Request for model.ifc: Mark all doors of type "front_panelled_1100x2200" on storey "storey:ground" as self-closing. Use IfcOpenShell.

First a look at what the model holds.

```python
import ifcopenshell
import ifcopenshell.util.element

model = ifcopenshell.open("model.ifc")
print(model.schema)
storey = next(s for s in model.by_type("IfcBuildingStorey") if s.Name == "storey:ground")
doors = [e for e in ifcopenshell.util.element.get_decomposition(storey) if e.is_a("IfcDoor")]
seen = {}
for e in doors:
    element_type = ifcopenshell.util.element.get_type(e)
    key = (element_type.Name if element_type != e and element_type else None, ifcopenshell.util.element.get_pset(e, "Pset_DoorCommon", "SelfClosing"))
    seen[key] = seen.get(key, 0) + 1
for (name, value), count in sorted(seen.items(), key=str):
    print(count, "x", name, "|", value)
```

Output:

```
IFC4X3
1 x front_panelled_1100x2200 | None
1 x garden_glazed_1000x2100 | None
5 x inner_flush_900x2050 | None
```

```python
import ifcopenshell
import ifcopenshell.api.pset
import ifcopenshell.util.element

model = ifcopenshell.open("model.ifc")

storey = next(s for s in model.by_type("IfcBuildingStorey") if s.Name == "storey:ground")
doors = [e for e in ifcopenshell.util.element.get_decomposition(storey) if e.is_a("IfcDoor")]

count = 0
for e in doors:
    element_type = ifcopenshell.util.element.get_type(e)
    if element_type in (None, e) or element_type.Name != "front_panelled_1100x2200":
        continue
    # add_pset returns the element's existing set when there is one.
    pset = ifcopenshell.api.pset.add_pset(model, product=e, name="Pset_DoorCommon")
    ifcopenshell.api.pset.edit_pset(model, pset=pset, properties={"SelfClosing": True})
    count += 1

print(count, "doors updated")

model.write("model-out.ifc")
```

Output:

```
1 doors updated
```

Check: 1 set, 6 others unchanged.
